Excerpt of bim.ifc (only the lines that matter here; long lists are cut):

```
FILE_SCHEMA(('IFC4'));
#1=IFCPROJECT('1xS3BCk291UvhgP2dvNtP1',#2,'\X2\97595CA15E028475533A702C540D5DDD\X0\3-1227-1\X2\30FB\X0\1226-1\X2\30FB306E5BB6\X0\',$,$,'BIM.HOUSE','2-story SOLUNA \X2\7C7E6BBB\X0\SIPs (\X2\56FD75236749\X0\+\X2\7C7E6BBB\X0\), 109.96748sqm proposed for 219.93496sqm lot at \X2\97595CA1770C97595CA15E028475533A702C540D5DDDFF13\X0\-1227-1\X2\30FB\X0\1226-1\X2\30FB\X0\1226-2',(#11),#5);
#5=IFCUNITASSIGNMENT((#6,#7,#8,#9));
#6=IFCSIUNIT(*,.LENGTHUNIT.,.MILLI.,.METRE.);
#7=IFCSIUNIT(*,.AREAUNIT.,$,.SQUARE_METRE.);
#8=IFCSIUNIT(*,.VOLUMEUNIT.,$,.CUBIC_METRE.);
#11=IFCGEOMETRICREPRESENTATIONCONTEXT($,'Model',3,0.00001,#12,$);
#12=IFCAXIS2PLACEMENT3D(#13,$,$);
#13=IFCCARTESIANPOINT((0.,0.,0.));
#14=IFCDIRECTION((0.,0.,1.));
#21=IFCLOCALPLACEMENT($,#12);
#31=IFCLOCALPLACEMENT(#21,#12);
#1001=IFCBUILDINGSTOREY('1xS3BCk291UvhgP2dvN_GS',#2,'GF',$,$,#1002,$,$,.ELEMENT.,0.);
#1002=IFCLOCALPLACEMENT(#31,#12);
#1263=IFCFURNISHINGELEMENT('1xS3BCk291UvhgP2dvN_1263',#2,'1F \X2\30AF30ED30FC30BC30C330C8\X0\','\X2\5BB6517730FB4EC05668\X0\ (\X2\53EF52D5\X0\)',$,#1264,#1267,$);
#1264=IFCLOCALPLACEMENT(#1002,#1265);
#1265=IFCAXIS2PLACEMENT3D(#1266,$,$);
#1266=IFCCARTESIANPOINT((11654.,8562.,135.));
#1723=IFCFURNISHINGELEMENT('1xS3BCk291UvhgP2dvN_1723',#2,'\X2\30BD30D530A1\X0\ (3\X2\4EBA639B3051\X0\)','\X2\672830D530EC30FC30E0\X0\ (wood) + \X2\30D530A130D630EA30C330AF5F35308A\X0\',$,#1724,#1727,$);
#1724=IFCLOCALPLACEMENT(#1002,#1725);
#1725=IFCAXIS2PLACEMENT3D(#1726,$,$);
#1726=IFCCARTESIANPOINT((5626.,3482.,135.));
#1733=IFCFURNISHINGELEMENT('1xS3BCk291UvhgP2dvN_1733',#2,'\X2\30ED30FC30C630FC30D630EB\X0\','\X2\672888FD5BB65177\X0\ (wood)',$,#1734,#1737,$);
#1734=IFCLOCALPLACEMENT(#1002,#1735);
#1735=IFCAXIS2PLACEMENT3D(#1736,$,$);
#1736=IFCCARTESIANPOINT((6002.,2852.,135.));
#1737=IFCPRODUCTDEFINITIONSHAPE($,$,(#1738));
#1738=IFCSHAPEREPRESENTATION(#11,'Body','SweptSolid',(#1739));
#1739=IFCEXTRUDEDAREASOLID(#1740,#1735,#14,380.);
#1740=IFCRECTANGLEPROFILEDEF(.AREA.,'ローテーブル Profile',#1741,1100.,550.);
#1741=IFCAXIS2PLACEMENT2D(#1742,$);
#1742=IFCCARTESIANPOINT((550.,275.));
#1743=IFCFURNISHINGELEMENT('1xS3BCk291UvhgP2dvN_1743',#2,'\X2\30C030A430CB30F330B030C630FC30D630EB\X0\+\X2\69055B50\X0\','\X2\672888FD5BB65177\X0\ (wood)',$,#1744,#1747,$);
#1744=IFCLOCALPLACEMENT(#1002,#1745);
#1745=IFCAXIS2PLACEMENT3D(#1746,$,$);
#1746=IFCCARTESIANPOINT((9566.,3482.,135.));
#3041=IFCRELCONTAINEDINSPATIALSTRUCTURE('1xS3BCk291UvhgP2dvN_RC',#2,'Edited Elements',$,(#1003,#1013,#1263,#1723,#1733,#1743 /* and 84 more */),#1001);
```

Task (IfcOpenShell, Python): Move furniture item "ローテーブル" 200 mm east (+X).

```python
import ifcopenshell
import ifcopenshell.api.geometry
import ifcopenshell.util.placement

model = ifcopenshell.open("bim.ifc")

item = model.by_id(1733)
matrix = ifcopenshell.util.placement.get_local_placement(item.ObjectPlacement)
matrix[0, 3] += 200.0
ifcopenshell.api.geometry.edit_object_placement(model, product=item, matrix=matrix, is_si=False)

print(ifcopenshell.util.placement.get_local_placement(item.ObjectPlacement).round(3) + 0.0)

model.write("bim_updated.ifc")
```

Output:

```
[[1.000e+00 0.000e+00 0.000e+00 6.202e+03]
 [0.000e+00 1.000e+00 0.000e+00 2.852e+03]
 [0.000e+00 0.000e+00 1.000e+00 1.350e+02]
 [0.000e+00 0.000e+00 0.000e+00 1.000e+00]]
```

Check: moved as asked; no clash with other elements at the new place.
